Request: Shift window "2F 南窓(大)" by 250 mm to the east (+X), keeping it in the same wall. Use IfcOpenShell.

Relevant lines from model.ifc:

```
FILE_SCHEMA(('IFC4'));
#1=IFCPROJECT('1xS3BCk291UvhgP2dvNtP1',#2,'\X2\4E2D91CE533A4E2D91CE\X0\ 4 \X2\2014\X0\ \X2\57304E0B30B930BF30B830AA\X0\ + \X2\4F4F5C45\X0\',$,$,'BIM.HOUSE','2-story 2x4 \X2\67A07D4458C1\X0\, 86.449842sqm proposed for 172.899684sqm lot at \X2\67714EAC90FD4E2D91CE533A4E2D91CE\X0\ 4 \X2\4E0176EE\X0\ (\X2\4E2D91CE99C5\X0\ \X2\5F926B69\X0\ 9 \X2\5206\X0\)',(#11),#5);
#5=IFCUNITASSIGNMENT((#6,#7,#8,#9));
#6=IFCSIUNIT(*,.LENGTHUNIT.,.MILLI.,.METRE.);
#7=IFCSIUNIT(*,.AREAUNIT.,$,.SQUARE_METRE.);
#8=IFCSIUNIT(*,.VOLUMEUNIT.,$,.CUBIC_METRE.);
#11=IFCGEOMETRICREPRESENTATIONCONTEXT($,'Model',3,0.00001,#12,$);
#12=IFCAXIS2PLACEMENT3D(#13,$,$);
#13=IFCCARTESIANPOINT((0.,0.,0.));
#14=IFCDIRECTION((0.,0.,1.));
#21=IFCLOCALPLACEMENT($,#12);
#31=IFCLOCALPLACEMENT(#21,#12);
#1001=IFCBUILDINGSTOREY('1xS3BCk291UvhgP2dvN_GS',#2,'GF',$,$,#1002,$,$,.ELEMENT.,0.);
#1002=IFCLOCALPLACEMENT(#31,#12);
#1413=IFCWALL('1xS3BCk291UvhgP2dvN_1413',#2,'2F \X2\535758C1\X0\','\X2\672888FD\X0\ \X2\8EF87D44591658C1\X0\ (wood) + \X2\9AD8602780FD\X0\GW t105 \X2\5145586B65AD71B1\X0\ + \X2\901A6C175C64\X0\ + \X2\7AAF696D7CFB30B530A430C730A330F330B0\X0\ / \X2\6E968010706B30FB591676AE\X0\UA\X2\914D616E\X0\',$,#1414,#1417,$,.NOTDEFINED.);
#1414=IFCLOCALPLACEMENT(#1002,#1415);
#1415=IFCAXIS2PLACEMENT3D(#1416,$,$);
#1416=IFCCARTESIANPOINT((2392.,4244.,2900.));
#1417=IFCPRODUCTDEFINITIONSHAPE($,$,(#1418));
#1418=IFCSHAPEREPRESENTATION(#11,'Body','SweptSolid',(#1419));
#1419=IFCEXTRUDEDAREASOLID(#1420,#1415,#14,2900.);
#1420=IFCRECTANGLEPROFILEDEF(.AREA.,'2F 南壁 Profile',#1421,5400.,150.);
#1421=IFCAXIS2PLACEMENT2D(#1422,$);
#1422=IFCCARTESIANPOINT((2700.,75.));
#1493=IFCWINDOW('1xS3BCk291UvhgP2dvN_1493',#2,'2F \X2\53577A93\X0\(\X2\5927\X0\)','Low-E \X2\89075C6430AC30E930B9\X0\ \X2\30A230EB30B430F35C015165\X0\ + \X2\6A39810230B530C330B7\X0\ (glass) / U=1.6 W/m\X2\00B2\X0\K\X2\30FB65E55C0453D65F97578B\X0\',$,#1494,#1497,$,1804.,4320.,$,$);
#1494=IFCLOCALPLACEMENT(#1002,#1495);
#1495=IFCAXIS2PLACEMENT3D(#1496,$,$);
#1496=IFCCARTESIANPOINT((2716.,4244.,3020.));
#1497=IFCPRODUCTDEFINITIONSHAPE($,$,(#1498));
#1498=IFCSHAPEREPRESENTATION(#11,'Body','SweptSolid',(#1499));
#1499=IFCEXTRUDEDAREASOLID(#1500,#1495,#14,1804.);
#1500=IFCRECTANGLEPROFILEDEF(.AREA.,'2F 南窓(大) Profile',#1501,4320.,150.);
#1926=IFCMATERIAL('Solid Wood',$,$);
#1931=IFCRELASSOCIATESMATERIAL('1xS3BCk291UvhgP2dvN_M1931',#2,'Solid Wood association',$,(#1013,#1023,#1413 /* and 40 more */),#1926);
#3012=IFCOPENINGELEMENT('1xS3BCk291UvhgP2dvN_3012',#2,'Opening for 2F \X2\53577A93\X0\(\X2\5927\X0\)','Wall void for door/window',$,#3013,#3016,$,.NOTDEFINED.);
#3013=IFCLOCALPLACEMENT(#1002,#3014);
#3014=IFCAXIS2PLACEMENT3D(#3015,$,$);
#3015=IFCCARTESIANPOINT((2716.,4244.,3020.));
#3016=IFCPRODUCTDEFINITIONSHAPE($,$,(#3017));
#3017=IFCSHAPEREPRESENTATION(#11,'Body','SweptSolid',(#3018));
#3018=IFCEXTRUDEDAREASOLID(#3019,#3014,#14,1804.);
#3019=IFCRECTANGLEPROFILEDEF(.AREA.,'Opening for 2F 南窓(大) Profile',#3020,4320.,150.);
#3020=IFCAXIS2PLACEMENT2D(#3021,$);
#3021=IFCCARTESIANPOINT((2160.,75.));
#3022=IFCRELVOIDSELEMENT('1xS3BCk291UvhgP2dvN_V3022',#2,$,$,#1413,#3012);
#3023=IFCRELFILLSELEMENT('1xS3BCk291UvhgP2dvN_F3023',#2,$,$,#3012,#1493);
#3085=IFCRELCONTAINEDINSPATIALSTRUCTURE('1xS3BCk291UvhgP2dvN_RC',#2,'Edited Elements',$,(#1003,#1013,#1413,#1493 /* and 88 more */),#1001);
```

```python
import ifcopenshell
import ifcopenshell.api.geometry
import ifcopenshell.util.placement

model = ifcopenshell.open("model.ifc")

window = model.by_guid("1xS3BCk291UvhgP2dvN_1493")
opening = window.FillsVoids[0].RelatingOpeningElement
wall = opening.VoidsElements[0].RelatingBuildingElement

wall_matrix = ifcopenshell.util.placement.get_local_placement(wall.ObjectPlacement)
shift = wall_matrix[:3, 0] * 250.0
before = ifcopenshell.util.placement.get_local_placement(window.ObjectPlacement)[:3, 3].copy()

# The window is not placed relative to its opening, so move both.
for product in (opening, window):
    matrix = ifcopenshell.util.placement.get_local_placement(product.ObjectPlacement)
    matrix[:3, 3] += shift
    ifcopenshell.api.geometry.edit_object_placement(model, product=product, matrix=matrix, is_si=False)

after = ifcopenshell.util.placement.get_local_placement(window.ObjectPlacement)[:3, 3]
print("window moved by", (after - before).round(3) + 0.0)

model.write("model_edited.ifc")
```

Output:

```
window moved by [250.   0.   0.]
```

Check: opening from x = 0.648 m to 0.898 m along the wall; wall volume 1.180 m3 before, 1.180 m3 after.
